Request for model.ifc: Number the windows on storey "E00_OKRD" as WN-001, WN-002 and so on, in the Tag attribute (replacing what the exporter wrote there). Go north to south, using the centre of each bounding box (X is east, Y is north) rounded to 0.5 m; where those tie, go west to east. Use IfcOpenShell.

First a look at what the model holds.

```python
import ifcopenshell
import ifcopenshell.util.element
import ifcopenshell.util.placement

model = ifcopenshell.open("model.ifc")
print(model.schema)
storey = next(s for s in model.by_type("IfcBuildingStorey") if s.Name == "E00_OKRD")
windows = [e for e in ifcopenshell.util.element.get_decomposition(storey) if e.is_a("IfcWindow")]
for e in sorted(windows, key=lambda e: e.id()):
    origin = ifcopenshell.util.placement.get_local_placement(e.ObjectPlacement)[:3, 3]
    print(e.id(), e.Tag, e.Name, origin.round(2) + 0.0, sep=" | ")
```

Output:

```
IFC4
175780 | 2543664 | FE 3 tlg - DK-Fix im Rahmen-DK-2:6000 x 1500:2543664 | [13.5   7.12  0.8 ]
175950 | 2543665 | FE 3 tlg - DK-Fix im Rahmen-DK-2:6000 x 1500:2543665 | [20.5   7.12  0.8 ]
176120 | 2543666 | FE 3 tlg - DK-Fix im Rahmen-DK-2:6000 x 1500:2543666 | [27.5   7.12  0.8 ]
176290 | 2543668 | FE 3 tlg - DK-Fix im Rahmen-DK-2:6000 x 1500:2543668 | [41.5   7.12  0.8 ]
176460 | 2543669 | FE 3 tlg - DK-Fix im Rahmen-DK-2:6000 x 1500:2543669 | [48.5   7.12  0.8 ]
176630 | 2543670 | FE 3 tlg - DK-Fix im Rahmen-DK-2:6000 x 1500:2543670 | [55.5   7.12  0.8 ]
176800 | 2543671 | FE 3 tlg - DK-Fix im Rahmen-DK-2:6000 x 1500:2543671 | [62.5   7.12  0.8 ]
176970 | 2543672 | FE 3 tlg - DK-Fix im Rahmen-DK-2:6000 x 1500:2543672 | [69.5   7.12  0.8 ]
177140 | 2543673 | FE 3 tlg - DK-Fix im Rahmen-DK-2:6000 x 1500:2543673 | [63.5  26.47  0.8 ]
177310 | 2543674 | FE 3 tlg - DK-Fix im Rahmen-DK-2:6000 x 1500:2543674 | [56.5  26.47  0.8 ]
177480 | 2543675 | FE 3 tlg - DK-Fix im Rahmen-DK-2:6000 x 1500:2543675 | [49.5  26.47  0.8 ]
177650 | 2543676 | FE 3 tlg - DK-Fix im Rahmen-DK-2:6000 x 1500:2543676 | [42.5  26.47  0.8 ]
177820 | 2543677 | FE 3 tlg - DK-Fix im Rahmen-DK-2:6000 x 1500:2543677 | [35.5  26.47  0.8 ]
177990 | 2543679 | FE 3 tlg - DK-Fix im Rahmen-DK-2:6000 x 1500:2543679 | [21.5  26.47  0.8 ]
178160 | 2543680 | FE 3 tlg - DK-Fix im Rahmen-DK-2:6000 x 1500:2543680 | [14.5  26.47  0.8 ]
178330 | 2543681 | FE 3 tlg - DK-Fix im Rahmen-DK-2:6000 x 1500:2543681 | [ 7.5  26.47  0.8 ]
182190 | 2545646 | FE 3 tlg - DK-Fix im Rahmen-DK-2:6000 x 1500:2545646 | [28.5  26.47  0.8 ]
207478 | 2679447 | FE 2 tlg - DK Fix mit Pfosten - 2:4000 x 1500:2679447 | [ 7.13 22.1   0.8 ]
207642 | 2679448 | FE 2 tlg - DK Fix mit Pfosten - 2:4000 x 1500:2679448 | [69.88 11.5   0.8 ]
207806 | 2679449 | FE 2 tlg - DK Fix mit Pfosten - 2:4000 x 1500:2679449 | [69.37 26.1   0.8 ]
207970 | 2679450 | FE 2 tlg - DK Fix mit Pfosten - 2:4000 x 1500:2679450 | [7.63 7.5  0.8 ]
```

```python
import ifcopenshell
import ifcopenshell.geom
import ifcopenshell.util.element
import ifcopenshell.util.shape

model = ifcopenshell.open("model.ifc")
settings = ifcopenshell.geom.settings()
settings.set("use-world-coords", True)


def centre(element):
    shape = ifcopenshell.geom.create_shape(settings, element)
    return ifcopenshell.util.shape.get_bbox_centroid(shape.geometry)


storey = next(s for s in model.by_type("IfcBuildingStorey") if s.Name == "E00_OKRD")
windows = [e for e in ifcopenshell.util.element.get_decomposition(storey) if e.is_a("IfcWindow")]

# Insertion points can sit at a corner or the storey origin, so sort by the geometry (in metres).
centres = {e: centre(e) for e in windows}
windows.sort(key=lambda e: (-round(centres[e][1] / 0.5), centres[e][0]))

for i, e in enumerate(windows, start=1):
    number = f"WN-0{i:02d}"
    e.Tag = number
    print(e.id(), number)

model.write("model_rev.ifc")
```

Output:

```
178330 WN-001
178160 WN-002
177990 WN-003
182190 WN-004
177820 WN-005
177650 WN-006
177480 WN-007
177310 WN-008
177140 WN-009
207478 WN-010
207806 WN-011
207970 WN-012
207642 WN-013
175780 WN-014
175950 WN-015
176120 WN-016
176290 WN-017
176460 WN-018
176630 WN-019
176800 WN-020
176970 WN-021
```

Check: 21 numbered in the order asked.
